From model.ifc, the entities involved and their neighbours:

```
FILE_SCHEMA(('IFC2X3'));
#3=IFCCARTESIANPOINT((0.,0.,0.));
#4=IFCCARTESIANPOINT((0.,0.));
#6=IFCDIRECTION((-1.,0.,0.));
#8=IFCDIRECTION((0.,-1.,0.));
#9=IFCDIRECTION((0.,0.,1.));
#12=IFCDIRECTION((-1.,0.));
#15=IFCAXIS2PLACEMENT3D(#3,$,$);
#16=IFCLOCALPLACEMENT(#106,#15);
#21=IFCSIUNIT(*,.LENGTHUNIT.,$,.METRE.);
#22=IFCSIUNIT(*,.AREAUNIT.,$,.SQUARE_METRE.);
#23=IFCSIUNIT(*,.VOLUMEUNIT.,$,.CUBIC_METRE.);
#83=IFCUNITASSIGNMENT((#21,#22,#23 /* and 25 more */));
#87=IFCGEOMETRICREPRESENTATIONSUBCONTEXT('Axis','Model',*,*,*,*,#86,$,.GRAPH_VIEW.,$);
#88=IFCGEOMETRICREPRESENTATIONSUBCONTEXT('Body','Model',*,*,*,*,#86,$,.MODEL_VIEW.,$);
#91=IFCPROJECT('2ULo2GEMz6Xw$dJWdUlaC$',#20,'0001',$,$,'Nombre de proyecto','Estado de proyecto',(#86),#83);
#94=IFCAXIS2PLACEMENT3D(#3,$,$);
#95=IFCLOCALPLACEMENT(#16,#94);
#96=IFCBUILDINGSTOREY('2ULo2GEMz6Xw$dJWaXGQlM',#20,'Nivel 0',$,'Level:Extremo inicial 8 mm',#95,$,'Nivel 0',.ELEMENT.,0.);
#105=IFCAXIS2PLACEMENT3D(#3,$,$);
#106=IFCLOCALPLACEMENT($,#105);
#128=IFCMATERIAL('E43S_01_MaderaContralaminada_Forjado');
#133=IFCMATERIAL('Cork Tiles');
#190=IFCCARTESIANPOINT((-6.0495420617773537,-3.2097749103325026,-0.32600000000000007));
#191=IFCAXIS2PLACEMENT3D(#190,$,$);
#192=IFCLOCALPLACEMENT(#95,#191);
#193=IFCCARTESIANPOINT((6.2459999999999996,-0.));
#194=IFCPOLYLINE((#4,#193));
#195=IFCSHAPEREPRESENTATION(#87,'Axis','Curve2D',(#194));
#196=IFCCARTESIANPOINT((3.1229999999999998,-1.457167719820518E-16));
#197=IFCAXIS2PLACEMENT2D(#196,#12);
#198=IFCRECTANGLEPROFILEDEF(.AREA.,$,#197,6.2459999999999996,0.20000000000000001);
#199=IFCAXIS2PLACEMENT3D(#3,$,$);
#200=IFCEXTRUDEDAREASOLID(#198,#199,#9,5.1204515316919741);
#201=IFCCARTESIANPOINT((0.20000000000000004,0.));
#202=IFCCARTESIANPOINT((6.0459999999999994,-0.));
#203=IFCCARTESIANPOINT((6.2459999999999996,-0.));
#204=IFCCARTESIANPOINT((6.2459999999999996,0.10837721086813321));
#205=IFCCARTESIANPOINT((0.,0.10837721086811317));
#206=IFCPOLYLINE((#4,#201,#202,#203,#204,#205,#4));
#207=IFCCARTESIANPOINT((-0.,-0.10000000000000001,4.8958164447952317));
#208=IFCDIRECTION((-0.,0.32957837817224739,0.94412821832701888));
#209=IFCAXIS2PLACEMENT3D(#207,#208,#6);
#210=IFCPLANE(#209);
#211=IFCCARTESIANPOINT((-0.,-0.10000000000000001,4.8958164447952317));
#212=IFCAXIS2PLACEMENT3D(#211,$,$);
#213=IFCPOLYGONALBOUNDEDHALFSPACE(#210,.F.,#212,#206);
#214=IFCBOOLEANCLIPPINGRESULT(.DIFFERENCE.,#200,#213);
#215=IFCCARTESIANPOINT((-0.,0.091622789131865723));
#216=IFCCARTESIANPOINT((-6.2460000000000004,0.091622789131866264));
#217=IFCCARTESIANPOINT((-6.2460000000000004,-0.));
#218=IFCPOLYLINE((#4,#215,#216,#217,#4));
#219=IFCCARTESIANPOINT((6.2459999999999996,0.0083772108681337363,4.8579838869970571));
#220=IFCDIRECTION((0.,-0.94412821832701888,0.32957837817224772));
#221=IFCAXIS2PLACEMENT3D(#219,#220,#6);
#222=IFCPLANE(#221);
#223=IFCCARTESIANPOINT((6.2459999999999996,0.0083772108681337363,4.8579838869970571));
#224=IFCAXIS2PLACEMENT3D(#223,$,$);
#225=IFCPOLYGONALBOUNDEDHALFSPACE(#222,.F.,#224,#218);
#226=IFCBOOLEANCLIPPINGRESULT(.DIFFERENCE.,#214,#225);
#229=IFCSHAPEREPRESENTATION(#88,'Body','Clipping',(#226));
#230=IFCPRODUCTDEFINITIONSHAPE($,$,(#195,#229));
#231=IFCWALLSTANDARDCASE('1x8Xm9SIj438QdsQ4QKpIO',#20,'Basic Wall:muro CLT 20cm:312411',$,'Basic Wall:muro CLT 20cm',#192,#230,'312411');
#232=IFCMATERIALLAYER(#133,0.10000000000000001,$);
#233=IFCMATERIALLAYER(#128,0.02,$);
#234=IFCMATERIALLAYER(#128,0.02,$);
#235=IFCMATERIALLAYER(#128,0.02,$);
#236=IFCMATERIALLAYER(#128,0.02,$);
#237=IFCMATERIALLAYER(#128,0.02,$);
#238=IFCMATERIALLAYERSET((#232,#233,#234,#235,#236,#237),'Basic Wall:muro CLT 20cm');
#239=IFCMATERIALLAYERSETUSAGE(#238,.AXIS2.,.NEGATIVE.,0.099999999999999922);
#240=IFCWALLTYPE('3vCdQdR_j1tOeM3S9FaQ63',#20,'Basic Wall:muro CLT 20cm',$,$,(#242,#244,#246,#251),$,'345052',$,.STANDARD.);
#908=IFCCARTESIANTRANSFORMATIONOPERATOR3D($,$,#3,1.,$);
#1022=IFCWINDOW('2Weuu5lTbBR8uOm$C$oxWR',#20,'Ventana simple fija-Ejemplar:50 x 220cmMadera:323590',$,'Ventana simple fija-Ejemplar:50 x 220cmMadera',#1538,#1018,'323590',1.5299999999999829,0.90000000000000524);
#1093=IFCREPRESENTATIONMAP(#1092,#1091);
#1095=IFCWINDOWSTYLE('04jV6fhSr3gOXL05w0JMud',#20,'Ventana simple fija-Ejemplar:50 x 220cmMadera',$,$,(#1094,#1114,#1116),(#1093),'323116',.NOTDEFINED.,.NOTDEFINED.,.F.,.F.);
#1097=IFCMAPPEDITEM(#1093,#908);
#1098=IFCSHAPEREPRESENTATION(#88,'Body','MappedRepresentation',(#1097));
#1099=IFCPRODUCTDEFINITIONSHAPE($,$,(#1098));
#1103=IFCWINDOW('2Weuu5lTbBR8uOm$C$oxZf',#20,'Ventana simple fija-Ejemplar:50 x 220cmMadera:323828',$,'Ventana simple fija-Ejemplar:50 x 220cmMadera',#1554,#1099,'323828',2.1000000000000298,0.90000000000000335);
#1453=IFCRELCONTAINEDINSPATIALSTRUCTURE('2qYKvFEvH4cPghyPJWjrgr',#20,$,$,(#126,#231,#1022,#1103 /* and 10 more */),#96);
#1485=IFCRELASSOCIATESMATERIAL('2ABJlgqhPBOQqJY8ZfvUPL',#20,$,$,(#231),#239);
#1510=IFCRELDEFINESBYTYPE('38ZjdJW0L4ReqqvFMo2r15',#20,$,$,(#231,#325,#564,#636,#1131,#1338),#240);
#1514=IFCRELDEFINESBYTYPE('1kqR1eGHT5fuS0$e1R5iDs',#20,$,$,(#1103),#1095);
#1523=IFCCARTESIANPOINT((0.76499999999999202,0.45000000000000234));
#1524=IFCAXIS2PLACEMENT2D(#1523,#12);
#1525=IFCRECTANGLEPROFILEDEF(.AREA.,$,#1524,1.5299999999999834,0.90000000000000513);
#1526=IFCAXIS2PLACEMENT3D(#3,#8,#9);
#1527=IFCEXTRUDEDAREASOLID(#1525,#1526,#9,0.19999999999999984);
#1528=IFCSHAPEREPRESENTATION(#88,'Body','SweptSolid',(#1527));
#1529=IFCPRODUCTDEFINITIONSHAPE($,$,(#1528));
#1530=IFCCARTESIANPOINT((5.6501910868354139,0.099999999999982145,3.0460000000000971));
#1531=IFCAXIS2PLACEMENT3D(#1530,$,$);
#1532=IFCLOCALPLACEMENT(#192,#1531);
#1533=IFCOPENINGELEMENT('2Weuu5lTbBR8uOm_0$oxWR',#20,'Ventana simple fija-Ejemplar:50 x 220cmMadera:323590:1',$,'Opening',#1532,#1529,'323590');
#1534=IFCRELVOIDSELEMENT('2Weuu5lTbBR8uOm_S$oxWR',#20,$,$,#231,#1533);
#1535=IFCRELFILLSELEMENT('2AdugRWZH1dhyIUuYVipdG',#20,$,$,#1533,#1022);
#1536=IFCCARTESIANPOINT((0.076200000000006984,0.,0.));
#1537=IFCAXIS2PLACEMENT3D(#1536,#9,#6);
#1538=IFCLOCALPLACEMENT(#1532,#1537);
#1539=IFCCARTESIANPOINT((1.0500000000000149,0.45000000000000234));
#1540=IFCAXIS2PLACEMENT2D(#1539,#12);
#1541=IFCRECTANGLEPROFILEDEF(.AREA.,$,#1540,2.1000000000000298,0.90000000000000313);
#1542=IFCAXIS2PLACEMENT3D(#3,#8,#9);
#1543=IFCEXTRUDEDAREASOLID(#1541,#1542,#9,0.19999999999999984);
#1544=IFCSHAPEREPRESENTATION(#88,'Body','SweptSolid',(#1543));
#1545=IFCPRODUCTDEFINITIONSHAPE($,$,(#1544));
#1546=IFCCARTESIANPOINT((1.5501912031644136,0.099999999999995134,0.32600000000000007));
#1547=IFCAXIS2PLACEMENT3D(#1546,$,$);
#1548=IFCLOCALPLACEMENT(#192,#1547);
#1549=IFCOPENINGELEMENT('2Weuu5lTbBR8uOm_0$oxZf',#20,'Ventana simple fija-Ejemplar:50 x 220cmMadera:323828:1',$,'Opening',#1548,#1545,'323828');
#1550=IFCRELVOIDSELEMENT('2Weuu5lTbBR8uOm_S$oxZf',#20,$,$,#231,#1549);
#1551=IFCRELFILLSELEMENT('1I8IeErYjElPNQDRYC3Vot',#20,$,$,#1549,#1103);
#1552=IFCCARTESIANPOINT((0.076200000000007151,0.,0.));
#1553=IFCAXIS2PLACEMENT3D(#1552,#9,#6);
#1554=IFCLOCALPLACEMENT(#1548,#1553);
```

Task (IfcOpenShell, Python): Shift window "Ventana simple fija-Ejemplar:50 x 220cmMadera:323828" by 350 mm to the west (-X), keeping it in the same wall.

```python
import ifcopenshell
import ifcopenshell.api.geometry
import ifcopenshell.util.placement
import ifcopenshell.util.unit

model = ifcopenshell.open("model.ifc")
unit_scale = ifcopenshell.util.unit.calculate_unit_scale(model)

window = model.by_id(1103)
opening = window.FillsVoids[0].RelatingOpeningElement
wall = opening.VoidsElements[0].RelatingBuildingElement

wall_matrix = ifcopenshell.util.placement.get_local_placement(wall.ObjectPlacement)
shift = wall_matrix[:3, 0] * -0.35 / unit_scale
before = ifcopenshell.util.placement.get_local_placement(window.ObjectPlacement)[:3, 3].copy()

# The window is placed relative to its opening, so it follows when the opening moves.
matrix = ifcopenshell.util.placement.get_local_placement(opening.ObjectPlacement)
matrix[:3, 3] += shift
ifcopenshell.api.geometry.edit_object_placement(
    model, product=opening, matrix=matrix, is_si=False, should_transform_children=True
)

after = ifcopenshell.util.placement.get_local_placement(window.ObjectPlacement)[:3, 3]
print("window moved by", (after - before).round(3) + 0.0)

model.write("model-out.ifc")
```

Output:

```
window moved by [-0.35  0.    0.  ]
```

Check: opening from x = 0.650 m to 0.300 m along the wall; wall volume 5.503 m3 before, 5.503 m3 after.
